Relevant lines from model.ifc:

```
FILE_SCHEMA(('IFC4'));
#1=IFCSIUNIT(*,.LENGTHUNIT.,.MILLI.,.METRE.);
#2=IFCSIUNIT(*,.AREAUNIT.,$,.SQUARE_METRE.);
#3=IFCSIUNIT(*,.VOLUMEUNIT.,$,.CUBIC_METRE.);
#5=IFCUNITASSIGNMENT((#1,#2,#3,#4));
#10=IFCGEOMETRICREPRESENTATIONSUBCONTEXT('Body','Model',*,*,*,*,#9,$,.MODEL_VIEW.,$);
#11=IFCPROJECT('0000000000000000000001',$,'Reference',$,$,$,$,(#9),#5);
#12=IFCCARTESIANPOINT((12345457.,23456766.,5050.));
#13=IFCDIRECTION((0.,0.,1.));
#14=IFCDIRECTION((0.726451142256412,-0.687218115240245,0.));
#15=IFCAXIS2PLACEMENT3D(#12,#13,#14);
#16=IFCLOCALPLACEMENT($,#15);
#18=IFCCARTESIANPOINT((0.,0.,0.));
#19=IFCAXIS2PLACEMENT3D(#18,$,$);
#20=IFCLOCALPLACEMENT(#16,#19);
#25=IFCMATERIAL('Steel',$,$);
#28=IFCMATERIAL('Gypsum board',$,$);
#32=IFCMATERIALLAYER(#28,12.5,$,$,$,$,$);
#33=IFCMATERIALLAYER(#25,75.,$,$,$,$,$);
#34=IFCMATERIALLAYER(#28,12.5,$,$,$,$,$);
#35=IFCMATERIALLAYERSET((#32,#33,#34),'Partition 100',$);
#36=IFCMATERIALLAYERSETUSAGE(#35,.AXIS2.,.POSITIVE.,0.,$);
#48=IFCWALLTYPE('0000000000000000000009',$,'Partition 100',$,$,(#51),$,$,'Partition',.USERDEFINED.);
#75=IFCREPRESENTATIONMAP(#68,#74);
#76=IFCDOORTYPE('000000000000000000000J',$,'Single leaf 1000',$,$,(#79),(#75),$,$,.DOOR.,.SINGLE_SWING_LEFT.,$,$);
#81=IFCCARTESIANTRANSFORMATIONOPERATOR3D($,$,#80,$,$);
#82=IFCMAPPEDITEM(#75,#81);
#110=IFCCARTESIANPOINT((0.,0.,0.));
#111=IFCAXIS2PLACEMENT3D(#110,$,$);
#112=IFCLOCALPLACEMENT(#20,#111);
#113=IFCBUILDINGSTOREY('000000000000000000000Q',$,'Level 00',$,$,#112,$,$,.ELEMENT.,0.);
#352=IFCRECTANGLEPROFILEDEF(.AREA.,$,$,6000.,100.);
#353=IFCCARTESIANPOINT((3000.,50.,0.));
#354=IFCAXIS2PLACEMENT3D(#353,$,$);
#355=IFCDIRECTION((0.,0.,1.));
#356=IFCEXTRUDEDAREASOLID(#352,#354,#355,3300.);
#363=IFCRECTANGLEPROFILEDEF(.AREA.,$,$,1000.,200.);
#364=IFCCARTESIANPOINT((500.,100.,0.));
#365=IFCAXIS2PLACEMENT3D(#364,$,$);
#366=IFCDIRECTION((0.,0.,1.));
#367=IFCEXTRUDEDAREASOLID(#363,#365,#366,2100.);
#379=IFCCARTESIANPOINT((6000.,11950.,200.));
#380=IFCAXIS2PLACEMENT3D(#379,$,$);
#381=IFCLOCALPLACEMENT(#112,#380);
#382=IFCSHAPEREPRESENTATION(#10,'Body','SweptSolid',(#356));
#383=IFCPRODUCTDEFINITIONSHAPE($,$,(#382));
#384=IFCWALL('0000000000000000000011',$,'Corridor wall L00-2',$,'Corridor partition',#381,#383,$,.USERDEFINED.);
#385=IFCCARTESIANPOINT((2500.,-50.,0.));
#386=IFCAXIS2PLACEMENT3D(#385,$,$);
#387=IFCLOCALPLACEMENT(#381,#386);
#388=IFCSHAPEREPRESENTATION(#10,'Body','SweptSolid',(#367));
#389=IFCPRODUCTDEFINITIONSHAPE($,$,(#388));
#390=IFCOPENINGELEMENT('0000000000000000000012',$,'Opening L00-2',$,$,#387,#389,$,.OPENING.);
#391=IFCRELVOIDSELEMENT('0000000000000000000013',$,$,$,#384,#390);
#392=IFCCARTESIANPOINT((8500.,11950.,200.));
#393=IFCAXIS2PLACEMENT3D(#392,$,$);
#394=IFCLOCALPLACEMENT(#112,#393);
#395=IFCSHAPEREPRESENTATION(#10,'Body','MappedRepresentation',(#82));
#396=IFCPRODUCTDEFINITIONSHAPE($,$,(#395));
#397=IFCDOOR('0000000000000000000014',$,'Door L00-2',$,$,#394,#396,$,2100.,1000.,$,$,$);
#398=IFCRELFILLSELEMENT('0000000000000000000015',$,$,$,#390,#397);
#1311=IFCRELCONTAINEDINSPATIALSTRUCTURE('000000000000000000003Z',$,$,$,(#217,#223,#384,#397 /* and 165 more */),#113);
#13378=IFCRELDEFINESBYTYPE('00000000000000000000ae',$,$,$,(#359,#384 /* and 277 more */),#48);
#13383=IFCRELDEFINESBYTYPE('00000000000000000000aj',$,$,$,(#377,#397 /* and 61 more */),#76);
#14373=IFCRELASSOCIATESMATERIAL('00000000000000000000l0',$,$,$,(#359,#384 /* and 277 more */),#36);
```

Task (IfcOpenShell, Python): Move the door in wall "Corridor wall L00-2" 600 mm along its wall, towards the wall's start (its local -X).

```python
import ifcopenshell
import ifcopenshell.api.geometry
import ifcopenshell.util.placement
import ifcopenshell.util.unit

model = ifcopenshell.open("model.ifc")
unit_scale = ifcopenshell.util.unit.calculate_unit_scale(model)

door = model.by_id(397)
opening = door.FillsVoids[0].RelatingOpeningElement
wall = opening.VoidsElements[0].RelatingBuildingElement

wall_matrix = ifcopenshell.util.placement.get_local_placement(wall.ObjectPlacement)
shift = wall_matrix[:3, 0] * -0.6 / unit_scale
before = ifcopenshell.util.placement.get_local_placement(door.ObjectPlacement)[:3, 3].copy()

# The door is not placed relative to its opening, so move both.
for product in (opening, door):
    matrix = ifcopenshell.util.placement.get_local_placement(product.ObjectPlacement)
    matrix[:3, 3] += shift
    ifcopenshell.api.geometry.edit_object_placement(model, product=product, matrix=matrix, is_si=False)

after = ifcopenshell.util.placement.get_local_placement(door.ObjectPlacement)[:3, 3]
print("door moved by", (after - before).round(3) + 0.0)

model.write("model_rev.ifc")
```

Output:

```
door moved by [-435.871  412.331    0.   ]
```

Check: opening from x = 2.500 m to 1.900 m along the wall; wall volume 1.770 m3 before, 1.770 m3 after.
